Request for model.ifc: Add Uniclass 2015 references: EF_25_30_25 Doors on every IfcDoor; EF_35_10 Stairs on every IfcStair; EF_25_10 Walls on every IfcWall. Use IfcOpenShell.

First a look at what the model holds.

```python
import ifcopenshell

model = ifcopenshell.open("model.ifc")
print(model.schema)
print("classifications:", [c.Name for c in model.by_type("IfcClassification")])
for ifc_class in ("IfcDoor", "IfcRoof", "IfcStair", "IfcWall", "IfcWindow"):
    print(ifc_class, len(model.by_type(ifc_class)))
```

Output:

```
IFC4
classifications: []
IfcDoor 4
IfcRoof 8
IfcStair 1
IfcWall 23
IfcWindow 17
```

```python
import ifcopenshell
import ifcopenshell.api.classification

model = ifcopenshell.open("model.ifc")

system = ifcopenshell.api.classification.add_classification(model, classification="Uniclass 2015")

codes = {
    "IfcDoor": ("EF_25_30_25", "Doors"),
    "IfcStair": ("EF_35_10", "Stairs"),
    "IfcWall": ("EF_25_10", "Walls"),
}
for ifc_class, (code, name) in codes.items():
    products = model.by_type(ifc_class)
    ifcopenshell.api.classification.add_reference(
        model, products=products, classification=system, identification=code, name=name
    )
    print(code, len(products))

model.write("model_v2.ifc")
```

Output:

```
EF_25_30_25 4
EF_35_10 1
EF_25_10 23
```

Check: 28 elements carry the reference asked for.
